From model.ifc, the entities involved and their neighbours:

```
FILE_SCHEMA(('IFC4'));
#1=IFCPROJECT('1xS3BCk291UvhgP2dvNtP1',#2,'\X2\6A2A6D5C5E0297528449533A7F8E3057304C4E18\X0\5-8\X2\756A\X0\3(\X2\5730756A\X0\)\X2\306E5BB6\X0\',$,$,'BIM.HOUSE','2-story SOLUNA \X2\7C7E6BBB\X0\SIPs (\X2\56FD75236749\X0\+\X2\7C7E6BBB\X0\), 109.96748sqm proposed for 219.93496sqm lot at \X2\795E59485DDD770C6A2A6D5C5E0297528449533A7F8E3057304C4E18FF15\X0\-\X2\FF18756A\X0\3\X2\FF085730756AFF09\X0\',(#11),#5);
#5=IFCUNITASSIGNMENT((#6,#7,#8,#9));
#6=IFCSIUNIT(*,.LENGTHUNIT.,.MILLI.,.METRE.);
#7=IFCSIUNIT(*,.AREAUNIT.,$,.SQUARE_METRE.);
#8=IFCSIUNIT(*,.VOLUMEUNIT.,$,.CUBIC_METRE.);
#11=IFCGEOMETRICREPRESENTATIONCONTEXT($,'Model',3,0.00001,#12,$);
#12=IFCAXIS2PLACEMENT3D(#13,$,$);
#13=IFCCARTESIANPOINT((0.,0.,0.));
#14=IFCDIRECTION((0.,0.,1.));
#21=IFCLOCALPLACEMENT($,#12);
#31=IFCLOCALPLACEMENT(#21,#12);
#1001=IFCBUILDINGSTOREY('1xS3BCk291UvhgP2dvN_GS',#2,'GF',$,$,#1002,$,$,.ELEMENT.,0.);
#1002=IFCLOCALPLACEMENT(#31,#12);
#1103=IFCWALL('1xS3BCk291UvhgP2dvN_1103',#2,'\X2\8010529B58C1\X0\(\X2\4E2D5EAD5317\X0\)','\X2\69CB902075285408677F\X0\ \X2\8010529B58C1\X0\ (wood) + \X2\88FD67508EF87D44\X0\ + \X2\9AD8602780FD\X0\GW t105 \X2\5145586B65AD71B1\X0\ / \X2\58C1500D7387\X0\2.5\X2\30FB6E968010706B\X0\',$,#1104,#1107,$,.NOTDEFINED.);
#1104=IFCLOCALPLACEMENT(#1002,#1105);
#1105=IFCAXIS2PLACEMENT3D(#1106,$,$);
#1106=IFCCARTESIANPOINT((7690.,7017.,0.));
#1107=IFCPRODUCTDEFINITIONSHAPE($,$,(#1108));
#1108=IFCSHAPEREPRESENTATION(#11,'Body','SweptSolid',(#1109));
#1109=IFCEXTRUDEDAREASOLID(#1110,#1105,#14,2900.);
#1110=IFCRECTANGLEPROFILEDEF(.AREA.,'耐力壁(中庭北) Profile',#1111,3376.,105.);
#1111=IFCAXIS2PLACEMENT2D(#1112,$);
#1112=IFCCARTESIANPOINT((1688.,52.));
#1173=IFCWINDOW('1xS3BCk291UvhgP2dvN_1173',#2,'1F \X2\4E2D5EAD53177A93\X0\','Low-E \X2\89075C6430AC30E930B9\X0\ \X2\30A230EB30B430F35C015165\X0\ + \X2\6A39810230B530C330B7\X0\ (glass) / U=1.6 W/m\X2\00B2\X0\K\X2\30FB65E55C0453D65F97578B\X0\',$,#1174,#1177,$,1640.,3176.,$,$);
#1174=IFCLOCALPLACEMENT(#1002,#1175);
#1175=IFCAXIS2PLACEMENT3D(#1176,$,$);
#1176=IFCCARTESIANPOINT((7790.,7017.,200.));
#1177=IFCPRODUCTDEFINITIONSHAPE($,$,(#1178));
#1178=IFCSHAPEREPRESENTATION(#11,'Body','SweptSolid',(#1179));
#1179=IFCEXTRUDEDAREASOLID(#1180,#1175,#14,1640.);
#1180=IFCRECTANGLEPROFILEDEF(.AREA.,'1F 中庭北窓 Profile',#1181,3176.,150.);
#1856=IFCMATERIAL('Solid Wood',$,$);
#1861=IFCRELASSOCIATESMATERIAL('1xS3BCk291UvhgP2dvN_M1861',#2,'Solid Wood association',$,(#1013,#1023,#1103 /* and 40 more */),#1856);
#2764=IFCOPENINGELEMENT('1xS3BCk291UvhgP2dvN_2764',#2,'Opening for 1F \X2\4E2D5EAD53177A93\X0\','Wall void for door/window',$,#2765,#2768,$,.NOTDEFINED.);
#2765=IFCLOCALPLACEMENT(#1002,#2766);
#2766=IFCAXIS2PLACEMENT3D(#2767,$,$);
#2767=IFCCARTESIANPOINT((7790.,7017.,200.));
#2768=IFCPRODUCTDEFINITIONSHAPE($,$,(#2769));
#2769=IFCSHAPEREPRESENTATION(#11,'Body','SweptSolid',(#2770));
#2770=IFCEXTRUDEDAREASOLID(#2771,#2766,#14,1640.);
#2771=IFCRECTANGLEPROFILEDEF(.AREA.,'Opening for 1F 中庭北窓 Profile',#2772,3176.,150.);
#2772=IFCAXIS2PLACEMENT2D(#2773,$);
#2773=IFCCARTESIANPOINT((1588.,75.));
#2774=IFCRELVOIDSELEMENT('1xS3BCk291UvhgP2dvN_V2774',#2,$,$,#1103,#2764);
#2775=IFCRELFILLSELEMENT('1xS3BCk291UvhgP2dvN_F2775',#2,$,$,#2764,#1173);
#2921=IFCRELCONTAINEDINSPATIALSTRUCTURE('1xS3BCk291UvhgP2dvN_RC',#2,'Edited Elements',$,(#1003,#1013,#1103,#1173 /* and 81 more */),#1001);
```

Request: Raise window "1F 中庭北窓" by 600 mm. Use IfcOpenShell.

```python
import numpy as np
import ifcopenshell
import ifcopenshell.api.geometry
import ifcopenshell.util.placement
import ifcopenshell.util.unit

model = ifcopenshell.open("model.ifc")
unit_scale = ifcopenshell.util.unit.calculate_unit_scale(model)

window = model.by_guid("1xS3BCk291UvhgP2dvN_1173")
opening = window.FillsVoids[0].RelatingOpeningElement
dz = 0.6 / unit_scale

shift = np.array([0.0, 0.0, dz])
# The window is not placed relative to its opening, so move both.
for product in (opening, window):
    matrix = ifcopenshell.util.placement.get_local_placement(product.ObjectPlacement)
    matrix[:3, 3] += shift
    ifcopenshell.api.geometry.edit_object_placement(model, product=product, matrix=matrix, is_si=False)

print(f"moved by {dz * unit_scale:+.3f} m")

model.write("model_v2.ifc")
```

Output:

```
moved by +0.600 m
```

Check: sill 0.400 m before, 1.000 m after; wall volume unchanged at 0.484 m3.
